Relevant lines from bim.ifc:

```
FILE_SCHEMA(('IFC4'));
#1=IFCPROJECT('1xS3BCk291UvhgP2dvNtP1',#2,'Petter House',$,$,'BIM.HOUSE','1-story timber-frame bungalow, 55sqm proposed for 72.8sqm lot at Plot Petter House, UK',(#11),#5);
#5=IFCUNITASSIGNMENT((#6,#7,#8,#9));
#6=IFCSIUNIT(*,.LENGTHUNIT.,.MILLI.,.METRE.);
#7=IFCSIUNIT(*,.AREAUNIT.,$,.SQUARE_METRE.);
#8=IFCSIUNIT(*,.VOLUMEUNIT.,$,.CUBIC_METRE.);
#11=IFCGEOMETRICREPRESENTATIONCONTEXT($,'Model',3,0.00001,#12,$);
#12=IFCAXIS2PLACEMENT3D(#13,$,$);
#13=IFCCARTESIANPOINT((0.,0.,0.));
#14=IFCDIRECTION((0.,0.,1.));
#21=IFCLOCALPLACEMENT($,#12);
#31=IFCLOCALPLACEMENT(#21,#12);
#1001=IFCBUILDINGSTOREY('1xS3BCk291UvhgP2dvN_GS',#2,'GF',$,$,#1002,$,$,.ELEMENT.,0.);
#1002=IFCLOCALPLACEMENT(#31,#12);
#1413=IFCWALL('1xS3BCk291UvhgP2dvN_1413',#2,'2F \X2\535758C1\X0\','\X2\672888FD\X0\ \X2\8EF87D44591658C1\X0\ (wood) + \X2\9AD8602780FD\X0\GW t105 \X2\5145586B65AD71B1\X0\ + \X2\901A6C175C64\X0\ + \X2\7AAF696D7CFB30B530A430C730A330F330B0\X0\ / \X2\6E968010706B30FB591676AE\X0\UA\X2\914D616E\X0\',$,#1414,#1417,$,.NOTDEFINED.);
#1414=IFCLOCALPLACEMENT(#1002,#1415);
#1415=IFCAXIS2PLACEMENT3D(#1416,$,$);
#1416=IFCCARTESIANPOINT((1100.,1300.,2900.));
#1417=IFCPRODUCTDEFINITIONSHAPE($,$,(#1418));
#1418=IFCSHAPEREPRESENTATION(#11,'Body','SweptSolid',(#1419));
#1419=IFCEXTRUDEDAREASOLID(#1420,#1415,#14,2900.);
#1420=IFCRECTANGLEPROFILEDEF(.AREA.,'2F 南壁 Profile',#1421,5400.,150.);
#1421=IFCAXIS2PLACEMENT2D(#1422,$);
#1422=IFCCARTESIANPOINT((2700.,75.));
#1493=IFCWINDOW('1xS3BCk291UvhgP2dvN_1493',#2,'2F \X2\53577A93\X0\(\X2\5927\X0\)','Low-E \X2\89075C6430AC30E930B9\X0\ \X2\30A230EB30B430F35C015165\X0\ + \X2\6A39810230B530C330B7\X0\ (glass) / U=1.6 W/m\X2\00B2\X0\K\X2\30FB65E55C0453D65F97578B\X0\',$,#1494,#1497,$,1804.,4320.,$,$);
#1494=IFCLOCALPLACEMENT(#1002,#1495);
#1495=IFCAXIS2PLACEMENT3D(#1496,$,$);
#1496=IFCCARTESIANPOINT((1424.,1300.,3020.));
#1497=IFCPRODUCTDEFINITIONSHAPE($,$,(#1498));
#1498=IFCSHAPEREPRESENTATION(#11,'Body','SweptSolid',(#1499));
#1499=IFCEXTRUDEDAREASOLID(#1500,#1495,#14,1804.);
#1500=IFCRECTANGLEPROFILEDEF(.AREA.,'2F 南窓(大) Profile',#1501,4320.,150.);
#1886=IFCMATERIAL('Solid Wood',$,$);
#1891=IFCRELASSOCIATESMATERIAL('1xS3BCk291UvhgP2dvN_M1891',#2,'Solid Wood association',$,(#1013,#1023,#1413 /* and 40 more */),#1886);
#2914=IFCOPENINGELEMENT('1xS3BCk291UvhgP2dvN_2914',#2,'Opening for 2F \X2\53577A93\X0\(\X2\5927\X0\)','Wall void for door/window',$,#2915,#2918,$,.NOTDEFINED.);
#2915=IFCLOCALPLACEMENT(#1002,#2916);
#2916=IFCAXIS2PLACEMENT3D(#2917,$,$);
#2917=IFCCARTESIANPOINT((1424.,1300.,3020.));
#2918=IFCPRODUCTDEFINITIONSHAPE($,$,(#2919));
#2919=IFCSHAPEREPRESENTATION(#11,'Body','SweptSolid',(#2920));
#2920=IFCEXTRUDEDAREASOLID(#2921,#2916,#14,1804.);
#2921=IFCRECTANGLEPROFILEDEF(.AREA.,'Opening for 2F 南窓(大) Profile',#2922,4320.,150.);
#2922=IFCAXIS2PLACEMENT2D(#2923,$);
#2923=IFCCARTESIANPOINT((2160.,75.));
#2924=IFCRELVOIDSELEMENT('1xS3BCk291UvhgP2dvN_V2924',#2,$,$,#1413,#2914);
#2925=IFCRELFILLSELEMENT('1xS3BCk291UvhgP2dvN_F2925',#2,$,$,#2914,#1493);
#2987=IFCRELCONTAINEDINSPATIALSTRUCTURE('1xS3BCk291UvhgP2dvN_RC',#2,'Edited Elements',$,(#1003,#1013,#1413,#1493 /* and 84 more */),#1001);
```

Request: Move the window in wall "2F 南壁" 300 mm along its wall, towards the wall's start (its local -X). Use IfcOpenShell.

```python
import ifcopenshell
import ifcopenshell.api.geometry
import ifcopenshell.util.placement
import ifcopenshell.util.unit

model = ifcopenshell.open("bim.ifc")
unit_scale = ifcopenshell.util.unit.calculate_unit_scale(model)

window = model.by_id(1493)
opening = window.FillsVoids[0].RelatingOpeningElement
wall = opening.VoidsElements[0].RelatingBuildingElement

wall_matrix = ifcopenshell.util.placement.get_local_placement(wall.ObjectPlacement)
shift = wall_matrix[:3, 0] * -0.3 / unit_scale
before = ifcopenshell.util.placement.get_local_placement(window.ObjectPlacement)[:3, 3].copy()

# The window is not placed relative to its opening, so move both.
for product in (opening, window):
    matrix = ifcopenshell.util.placement.get_local_placement(product.ObjectPlacement)
    matrix[:3, 3] += shift
    ifcopenshell.api.geometry.edit_object_placement(model, product=product, matrix=matrix, is_si=False)

after = ifcopenshell.util.placement.get_local_placement(window.ObjectPlacement)[:3, 3]
print("window moved by", (after - before).round(3) + 0.0)

model.write("bim_updated.ifc")
```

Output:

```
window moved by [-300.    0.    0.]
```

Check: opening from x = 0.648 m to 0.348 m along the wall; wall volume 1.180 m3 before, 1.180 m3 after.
